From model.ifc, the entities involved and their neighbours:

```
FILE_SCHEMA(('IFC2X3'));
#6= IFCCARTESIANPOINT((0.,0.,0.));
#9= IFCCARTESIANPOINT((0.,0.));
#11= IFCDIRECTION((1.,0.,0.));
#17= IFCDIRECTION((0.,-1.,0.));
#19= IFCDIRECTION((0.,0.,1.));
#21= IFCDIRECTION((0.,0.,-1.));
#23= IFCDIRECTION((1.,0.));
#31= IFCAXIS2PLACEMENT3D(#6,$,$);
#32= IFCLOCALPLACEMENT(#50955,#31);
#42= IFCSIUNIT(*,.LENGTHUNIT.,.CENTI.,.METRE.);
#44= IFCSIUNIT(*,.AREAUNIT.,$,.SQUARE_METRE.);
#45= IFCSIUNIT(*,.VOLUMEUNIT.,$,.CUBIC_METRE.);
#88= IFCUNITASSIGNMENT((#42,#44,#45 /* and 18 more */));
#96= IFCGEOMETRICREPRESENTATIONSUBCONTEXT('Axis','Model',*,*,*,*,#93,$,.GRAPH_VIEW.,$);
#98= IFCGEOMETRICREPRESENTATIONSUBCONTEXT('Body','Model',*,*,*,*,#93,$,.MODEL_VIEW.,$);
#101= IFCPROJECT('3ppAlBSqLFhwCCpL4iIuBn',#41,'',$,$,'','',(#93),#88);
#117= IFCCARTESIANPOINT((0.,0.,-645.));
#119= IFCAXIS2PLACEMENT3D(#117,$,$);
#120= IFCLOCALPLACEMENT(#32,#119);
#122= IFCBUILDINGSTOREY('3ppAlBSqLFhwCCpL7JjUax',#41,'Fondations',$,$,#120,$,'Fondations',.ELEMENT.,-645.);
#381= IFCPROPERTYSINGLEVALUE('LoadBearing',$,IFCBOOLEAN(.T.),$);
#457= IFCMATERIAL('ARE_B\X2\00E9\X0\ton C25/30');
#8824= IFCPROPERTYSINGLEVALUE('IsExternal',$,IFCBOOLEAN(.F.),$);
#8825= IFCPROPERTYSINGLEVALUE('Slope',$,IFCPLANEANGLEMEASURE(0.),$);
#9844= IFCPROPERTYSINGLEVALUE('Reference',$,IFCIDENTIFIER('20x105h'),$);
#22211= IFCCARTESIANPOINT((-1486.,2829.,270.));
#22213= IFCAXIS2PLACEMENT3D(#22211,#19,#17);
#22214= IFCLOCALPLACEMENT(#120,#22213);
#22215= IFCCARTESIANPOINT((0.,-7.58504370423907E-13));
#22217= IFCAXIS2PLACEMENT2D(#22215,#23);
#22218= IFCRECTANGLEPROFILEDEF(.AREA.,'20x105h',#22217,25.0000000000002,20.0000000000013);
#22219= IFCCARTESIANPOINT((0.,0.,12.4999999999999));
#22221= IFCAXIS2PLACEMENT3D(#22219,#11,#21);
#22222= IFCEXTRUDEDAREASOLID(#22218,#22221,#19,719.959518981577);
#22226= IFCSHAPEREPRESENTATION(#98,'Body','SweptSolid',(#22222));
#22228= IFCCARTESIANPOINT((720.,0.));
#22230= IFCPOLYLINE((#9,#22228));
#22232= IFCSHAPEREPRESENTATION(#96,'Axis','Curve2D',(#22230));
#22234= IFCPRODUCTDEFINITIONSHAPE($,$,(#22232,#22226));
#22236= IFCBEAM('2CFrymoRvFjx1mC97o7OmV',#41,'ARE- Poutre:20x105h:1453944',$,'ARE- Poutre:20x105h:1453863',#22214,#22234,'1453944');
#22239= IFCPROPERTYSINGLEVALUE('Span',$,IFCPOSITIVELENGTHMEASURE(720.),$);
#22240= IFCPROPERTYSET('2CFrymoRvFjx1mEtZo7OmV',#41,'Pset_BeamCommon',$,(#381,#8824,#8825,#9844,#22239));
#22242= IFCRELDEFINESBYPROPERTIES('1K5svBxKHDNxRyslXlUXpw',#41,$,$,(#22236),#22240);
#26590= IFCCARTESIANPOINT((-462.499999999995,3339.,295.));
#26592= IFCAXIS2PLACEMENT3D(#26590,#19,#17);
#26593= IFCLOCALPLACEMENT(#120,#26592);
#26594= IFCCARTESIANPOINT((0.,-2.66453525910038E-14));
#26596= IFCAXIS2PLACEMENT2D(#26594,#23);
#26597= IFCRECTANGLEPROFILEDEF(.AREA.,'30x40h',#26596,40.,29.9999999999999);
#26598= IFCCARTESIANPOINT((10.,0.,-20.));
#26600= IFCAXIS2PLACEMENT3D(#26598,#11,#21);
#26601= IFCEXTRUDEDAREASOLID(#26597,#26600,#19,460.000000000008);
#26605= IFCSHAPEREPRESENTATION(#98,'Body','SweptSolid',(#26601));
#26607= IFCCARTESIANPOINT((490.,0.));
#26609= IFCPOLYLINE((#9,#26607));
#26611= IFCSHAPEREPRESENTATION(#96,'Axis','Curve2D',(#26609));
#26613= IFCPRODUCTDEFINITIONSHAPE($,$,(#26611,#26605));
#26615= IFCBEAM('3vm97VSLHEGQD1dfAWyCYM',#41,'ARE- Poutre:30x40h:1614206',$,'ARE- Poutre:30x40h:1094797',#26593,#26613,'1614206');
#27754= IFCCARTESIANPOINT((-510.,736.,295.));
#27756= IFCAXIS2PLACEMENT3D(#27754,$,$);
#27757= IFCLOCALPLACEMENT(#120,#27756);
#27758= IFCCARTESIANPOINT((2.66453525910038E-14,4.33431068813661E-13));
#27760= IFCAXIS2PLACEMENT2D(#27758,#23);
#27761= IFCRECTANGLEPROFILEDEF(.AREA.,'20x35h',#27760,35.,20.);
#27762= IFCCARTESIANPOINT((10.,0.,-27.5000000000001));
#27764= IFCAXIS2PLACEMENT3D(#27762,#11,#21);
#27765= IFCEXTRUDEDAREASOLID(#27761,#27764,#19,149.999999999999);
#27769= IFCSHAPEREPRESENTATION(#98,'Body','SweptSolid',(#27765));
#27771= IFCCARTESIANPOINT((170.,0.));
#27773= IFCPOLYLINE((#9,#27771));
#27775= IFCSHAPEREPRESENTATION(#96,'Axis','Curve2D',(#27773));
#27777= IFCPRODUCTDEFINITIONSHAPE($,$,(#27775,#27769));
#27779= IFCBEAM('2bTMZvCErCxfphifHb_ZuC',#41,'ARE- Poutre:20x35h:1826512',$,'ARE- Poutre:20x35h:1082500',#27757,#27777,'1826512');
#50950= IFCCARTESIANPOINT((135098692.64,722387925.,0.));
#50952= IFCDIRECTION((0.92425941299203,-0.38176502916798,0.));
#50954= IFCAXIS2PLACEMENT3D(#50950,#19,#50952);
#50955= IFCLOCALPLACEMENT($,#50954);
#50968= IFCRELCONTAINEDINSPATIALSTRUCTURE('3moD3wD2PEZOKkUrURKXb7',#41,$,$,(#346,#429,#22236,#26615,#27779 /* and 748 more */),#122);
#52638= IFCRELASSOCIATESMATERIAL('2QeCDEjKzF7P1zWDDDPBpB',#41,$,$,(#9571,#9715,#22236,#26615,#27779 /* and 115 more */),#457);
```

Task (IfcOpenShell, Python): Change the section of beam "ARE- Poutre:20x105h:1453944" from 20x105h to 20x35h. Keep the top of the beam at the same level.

```python
import ifcopenshell
import ifcopenshell.api.pset
import ifcopenshell.util.element
import ifcopenshell.util.representation

model = ifcopenshell.open("model.ifc")

member = model.by_id(22236)
source = next(p for p in model.by_type("IfcRectangleProfileDef") if p.ProfileName == "20x35h")

body = ifcopenshell.util.representation.get_representation(member, "Model", "Body")
solid = body.Items[0]
old_profile = solid.SweptArea

# Copy the section's sizes but keep this member's own profile position.
profile = ifcopenshell.util.element.copy(model, source)
# Profiles are centred, so shift by half the change in depth to hold the top.
shift = (old_profile.XDim - profile.XDim) / 2
x, y = old_profile.Position.Location.Coordinates
up = (-1.0, 0.0)  # upwards, in the solid's own plane
location = model.createIfcCartesianPoint((x + up[0] * shift, y + up[1] * shift))
profile.Position = model.createIfcAxis2Placement2D(location, old_profile.Position.RefDirection)
solid.SweptArea = profile
if not model.get_total_inverses(old_profile):
    ifcopenshell.util.element.remove_deep2(model, old_profile)
member.Name = member.Name.replace("20x105h", "20x35h")
member.ObjectType = member.ObjectType.replace("20x105h", "20x35h")
pset = model.by_id(ifcopenshell.util.element.get_pset(member, "Pset_BeamCommon", should_inherit=False)["id"])
ifcopenshell.api.pset.edit_pset(model, pset=pset, properties={"Reference": "20x35h"})

print(solid.SweptArea)

model.write("model_edited.ifc")
```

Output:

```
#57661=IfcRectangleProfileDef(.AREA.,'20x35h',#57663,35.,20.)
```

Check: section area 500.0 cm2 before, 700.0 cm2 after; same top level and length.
